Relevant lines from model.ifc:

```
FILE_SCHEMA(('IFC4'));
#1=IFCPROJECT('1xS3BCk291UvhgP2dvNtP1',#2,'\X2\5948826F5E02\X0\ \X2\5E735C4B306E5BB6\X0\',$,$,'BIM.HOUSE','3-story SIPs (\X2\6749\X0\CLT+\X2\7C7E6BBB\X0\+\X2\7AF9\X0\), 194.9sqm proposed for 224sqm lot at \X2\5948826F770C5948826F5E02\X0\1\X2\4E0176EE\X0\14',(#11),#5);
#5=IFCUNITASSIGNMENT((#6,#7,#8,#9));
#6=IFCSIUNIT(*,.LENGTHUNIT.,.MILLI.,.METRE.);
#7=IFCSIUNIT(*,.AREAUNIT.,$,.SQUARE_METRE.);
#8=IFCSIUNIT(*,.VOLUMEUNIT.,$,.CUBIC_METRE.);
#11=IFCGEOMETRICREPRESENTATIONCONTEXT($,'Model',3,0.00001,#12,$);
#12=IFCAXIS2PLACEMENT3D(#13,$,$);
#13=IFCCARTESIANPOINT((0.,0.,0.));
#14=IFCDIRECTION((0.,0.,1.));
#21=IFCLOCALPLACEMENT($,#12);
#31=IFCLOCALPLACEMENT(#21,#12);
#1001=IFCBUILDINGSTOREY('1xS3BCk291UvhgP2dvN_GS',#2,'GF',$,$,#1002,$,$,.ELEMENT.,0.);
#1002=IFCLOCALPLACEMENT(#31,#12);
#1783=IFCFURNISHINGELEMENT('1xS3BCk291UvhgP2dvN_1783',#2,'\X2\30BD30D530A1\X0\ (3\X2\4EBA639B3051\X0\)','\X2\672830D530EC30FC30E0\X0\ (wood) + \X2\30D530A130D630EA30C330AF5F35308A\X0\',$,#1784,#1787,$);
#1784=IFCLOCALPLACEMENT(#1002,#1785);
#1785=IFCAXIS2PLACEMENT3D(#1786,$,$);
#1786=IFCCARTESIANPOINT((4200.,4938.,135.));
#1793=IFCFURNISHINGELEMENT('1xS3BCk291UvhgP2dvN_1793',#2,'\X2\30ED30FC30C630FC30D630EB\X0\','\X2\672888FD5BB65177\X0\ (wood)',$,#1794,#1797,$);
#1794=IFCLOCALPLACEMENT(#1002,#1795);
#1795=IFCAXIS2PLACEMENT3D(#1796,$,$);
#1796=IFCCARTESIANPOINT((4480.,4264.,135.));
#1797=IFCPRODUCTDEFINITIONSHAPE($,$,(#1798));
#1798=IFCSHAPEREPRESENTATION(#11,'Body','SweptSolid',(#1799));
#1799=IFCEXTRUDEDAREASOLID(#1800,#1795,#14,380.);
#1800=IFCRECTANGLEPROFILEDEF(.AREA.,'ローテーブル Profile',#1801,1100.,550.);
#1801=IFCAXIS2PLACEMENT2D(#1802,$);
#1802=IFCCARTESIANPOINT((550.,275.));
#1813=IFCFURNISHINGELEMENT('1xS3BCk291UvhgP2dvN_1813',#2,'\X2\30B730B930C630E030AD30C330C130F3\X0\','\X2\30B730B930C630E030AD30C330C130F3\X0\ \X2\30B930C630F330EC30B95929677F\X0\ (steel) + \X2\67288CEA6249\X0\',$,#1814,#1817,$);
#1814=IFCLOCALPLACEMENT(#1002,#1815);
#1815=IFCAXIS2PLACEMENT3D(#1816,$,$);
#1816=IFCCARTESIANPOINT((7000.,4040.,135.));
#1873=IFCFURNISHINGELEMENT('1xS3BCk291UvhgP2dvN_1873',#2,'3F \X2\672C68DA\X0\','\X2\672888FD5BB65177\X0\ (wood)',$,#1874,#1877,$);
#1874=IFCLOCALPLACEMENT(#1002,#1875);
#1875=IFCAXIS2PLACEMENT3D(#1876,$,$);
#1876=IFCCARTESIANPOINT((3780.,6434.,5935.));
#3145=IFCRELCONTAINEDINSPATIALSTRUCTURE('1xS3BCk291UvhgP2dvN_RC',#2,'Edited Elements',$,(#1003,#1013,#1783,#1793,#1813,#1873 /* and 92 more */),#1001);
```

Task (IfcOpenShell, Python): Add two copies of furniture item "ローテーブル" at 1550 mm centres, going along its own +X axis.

```python
import ifcopenshell
import ifcopenshell.api.geometry
import ifcopenshell.api.root
import ifcopenshell.util.element
import ifcopenshell.util.placement
import ifcopenshell.util.unit

model = ifcopenshell.open("model.ifc")
unit_scale = ifcopenshell.util.unit.calculate_unit_scale(model)


def reuse_history(source, copy):
    """copy_class also copies each property set's owner history, people and application; keep the originals."""
    for rel in copy.IsDefinedBy:
        if rel.is_a("IfcRelDefinesByProperties") and (history := rel.RelatingPropertyDefinition.OwnerHistory):
            rel.RelatingPropertyDefinition.OwnerHistory = source.OwnerHistory
            ifcopenshell.util.element.remove_deep2(model, history)


source = model.by_id(1793)
base = ifcopenshell.util.placement.get_local_placement(source.ObjectPlacement)
step = base[:3, 0] * 1.55 / unit_scale

for i in range(1, 3):
    copy = ifcopenshell.api.root.copy_class(model, product=source)
    copy.Representation = ifcopenshell.util.element.copy_deep(
        model, source.Representation, exclude=["IfcGeometricRepresentationContext", "IfcRepresentationMap"]
    )
    reuse_history(source, copy)
    matrix = base.copy()
    matrix[:3, 3] += i * step
    print("added at", matrix[:3, 3].round(3) + 0.0)
    ifcopenshell.api.geometry.edit_object_placement(model, product=copy, matrix=matrix, is_si=False)

model.write("model_updated.ifc")
```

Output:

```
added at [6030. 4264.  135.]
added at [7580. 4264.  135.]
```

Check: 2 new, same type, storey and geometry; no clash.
